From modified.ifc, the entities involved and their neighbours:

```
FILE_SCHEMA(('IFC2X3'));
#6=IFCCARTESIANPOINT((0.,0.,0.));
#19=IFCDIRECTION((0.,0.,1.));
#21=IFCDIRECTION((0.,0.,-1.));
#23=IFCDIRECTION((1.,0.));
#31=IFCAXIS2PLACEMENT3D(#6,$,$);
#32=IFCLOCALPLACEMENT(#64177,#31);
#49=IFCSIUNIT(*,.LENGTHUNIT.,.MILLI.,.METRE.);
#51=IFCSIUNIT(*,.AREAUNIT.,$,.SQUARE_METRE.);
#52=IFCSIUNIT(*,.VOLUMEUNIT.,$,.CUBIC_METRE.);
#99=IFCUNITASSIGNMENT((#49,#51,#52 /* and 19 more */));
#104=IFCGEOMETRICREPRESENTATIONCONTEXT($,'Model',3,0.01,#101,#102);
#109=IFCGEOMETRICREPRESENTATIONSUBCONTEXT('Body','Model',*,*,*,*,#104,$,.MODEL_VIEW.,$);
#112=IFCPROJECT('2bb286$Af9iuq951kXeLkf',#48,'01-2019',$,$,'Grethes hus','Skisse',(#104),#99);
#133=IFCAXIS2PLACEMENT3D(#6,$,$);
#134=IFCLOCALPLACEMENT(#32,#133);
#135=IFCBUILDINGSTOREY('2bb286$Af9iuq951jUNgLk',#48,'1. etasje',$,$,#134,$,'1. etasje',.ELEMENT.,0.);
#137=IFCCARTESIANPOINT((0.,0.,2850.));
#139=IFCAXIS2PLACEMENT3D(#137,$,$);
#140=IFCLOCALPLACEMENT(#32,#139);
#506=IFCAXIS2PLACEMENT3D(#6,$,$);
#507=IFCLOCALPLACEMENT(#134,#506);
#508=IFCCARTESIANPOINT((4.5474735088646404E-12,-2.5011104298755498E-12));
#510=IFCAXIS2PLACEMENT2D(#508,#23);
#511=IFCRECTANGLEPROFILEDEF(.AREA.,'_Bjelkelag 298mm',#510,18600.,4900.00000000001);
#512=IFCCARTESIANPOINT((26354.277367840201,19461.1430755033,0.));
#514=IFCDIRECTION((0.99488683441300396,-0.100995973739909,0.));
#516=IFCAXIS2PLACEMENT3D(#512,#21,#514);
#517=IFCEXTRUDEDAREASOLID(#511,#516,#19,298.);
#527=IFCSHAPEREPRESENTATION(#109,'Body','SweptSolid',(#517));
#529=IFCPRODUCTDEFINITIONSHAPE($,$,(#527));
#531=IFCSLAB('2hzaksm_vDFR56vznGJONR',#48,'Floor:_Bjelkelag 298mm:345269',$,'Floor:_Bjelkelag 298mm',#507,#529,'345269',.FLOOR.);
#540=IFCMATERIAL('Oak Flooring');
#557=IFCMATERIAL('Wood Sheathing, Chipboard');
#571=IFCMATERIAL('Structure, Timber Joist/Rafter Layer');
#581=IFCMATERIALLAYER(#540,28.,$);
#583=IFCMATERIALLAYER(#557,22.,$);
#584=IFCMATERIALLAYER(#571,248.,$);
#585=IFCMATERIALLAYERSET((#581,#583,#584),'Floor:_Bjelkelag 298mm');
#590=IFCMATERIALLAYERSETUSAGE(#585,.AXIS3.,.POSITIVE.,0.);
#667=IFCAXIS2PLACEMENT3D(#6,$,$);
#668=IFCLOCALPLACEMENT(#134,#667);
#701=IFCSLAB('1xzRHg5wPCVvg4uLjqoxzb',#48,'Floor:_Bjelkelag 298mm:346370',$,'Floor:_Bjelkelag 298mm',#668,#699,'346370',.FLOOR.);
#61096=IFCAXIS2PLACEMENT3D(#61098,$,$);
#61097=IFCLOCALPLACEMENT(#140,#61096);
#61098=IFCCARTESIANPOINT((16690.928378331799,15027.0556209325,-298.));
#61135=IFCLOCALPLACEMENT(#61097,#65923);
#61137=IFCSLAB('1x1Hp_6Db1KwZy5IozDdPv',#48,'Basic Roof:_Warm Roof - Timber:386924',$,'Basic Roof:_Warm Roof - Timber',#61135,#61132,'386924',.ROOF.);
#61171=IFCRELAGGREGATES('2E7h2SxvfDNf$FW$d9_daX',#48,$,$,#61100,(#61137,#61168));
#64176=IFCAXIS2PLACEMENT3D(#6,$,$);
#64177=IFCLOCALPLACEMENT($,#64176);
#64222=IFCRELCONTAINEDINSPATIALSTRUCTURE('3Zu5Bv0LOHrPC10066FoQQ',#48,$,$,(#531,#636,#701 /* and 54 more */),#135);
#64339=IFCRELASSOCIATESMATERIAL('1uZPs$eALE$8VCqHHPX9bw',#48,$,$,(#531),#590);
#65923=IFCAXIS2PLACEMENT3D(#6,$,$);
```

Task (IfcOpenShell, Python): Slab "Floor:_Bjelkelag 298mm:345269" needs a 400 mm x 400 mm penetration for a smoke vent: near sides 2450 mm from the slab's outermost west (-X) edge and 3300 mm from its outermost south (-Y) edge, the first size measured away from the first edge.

```python
import numpy as np
import ifcopenshell
import ifcopenshell.api.feature
import ifcopenshell.api.geometry
import ifcopenshell.api.root
import ifcopenshell.geom
import ifcopenshell.util.placement
import ifcopenshell.util.representation
import ifcopenshell.util.shape
import ifcopenshell.util.unit

model = ifcopenshell.open("modified.ifc")
unit_scale = ifcopenshell.util.unit.calculate_unit_scale(model)
settings = ifcopenshell.geom.settings()


def volume(element):
    """Net volume in cubic metres, openings subtracted."""
    shape = ifcopenshell.geom.create_shape(settings, element)
    return ifcopenshell.util.shape.get_volume(shape.geometry)


slab = model.by_id(531)
before = volume(slab)

# Extent in the slab's own axes, in metres. The edges named are its -X and -Y sides.
slab_shape = ifcopenshell.geom.create_shape(settings, slab)
vertices = ifcopenshell.util.shape.get_vertices(slab_shape.geometry)
x_min, y_min, bottom = vertices.min(axis=0)
top = vertices[:, 2].max()

opening = ifcopenshell.api.root.create_entity(model, ifc_class="IfcOpeningElement", name="Smoke vent opening")
context = ifcopenshell.util.representation.get_context(model, "Model", "Body", "MODEL_VIEW")
width, depth = 0.4, 0.4
outline = [(0.0, 0.0), (width, 0.0), (width, depth), (0.0, depth), (0.0, 0.0)]
# Overshoot both faces by 50 mm so the cut is clean.
shape = ifcopenshell.api.geometry.add_slab_representation(
    model, context=context, depth=top - bottom + 0.1, polyline=outline
)
ifcopenshell.api.geometry.assign_representation(model, product=opening, representation=shape)

matrix = ifcopenshell.util.placement.get_local_placement(slab.ObjectPlacement)
matrix[:, 3] = matrix @ np.append(np.array([x_min + 2.45, y_min + 3.3, bottom - 0.05]) / unit_scale, 1.0)
ifcopenshell.api.geometry.edit_object_placement(model, product=opening, matrix=matrix, is_si=False)
ifcopenshell.api.feature.add_feature(model, feature=opening, element=slab)

after = volume(slab)

print(f"slab volume {before:.3f} -> {after:.3f} m3")

model.write("modified-out.ifc")
```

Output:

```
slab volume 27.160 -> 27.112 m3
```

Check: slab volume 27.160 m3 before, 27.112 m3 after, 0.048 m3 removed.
